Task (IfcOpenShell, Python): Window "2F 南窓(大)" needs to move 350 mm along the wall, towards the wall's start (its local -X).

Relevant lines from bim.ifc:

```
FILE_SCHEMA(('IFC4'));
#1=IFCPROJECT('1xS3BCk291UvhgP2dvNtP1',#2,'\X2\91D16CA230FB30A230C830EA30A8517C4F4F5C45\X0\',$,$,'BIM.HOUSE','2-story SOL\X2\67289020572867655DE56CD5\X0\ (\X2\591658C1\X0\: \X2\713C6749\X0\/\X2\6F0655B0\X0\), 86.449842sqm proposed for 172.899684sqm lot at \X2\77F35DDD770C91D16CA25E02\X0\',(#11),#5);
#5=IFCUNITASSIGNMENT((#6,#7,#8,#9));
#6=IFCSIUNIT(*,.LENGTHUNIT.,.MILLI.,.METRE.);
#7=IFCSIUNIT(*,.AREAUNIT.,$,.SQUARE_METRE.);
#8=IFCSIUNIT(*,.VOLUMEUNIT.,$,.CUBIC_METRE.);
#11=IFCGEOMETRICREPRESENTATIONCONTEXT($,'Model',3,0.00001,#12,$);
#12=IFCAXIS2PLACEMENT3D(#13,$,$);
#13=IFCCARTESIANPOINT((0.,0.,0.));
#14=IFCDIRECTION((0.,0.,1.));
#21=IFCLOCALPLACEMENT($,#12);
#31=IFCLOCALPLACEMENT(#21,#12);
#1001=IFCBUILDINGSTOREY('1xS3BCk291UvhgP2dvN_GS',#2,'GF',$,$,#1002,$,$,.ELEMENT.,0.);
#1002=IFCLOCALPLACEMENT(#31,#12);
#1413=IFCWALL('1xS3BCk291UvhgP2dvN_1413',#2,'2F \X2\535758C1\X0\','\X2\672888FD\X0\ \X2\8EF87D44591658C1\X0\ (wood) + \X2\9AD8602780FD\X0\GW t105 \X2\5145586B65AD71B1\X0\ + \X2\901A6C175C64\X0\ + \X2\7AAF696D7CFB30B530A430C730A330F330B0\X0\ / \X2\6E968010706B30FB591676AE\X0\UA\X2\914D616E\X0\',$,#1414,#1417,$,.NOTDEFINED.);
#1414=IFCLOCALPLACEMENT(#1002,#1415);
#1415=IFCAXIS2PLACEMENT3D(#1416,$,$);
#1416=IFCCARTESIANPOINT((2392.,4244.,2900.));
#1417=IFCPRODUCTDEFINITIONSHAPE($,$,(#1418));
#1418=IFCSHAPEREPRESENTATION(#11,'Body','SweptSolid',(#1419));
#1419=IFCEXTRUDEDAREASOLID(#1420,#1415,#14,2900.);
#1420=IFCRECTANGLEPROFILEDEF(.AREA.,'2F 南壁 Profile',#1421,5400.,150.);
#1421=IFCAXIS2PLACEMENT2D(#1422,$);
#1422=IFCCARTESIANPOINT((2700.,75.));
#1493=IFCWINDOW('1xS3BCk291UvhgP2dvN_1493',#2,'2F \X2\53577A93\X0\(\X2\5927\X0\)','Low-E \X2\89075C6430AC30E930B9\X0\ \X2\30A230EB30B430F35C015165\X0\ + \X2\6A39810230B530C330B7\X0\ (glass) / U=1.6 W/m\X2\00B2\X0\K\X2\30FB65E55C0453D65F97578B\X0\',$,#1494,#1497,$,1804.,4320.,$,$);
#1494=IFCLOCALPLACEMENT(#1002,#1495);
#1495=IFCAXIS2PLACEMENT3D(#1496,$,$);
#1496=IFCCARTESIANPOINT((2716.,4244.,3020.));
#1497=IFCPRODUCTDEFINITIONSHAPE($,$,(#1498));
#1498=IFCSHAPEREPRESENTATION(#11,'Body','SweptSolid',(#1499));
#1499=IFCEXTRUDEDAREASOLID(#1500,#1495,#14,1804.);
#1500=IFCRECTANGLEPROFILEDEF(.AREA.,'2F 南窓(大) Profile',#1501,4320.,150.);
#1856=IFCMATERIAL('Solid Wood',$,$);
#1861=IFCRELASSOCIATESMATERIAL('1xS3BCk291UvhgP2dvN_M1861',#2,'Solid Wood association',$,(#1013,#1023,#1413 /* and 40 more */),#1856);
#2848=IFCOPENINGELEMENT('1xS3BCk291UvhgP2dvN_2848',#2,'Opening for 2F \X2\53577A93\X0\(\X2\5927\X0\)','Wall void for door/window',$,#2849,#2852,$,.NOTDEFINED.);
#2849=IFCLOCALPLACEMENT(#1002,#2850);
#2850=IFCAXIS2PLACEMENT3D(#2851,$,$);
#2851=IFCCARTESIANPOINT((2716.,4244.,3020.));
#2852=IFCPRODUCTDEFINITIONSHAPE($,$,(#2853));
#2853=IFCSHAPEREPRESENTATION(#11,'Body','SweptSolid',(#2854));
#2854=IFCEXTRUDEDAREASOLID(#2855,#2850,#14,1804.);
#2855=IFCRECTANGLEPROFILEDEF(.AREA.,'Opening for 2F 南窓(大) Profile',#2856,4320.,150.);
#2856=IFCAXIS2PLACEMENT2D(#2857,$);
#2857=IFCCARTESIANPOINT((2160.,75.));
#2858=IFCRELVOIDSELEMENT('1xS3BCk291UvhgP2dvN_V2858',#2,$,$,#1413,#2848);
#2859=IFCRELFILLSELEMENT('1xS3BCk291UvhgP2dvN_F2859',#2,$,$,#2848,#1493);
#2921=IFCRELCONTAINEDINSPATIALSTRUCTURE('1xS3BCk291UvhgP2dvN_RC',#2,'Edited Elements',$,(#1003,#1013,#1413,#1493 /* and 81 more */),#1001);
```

```python
import ifcopenshell
import ifcopenshell.api.geometry
import ifcopenshell.util.placement

model = ifcopenshell.open("bim.ifc")

window = model.by_guid("1xS3BCk291UvhgP2dvN_1493")
opening = window.FillsVoids[0].RelatingOpeningElement
wall = opening.VoidsElements[0].RelatingBuildingElement

wall_matrix = ifcopenshell.util.placement.get_local_placement(wall.ObjectPlacement)
shift = wall_matrix[:3, 0] * -350.0
before = ifcopenshell.util.placement.get_local_placement(window.ObjectPlacement)[:3, 3].copy()

# The window is not placed relative to its opening, so move both.
for product in (opening, window):
    matrix = ifcopenshell.util.placement.get_local_placement(product.ObjectPlacement)
    matrix[:3, 3] += shift
    ifcopenshell.api.geometry.edit_object_placement(model, product=product, matrix=matrix, is_si=False)

after = ifcopenshell.util.placement.get_local_placement(window.ObjectPlacement)[:3, 3]
print("window moved by", (after - before).round(3) + 0.0)

model.write("bim_updated.ifc")
```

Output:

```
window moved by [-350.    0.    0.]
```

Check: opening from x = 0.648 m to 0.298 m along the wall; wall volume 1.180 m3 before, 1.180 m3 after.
